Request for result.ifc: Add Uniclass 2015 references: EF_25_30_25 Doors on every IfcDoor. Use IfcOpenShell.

First a look at what the model holds.

```python
import ifcopenshell

model = ifcopenshell.open("result.ifc")
print(model.schema)
print("classifications:", [c.Name for c in model.by_type("IfcClassification")])
for ifc_class in ("IfcDoor", "IfcRoof", "IfcStair", "IfcWall", "IfcWindow"):
    print(ifc_class, len(model.by_type(ifc_class)))
```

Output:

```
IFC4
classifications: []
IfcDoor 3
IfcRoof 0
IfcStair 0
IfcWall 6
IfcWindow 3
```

```python
import ifcopenshell
import ifcopenshell.api.classification

model = ifcopenshell.open("result.ifc")

system = ifcopenshell.api.classification.add_classification(model, classification="Uniclass 2015")

codes = {
    "IfcDoor": ("EF_25_30_25", "Doors"),
}
for ifc_class, (code, name) in codes.items():
    products = model.by_type(ifc_class)
    ifcopenshell.api.classification.add_reference(
        model, products=products, classification=system, identification=code, name=name
    )
    print(code, len(products))

model.write("result_updated.ifc")
```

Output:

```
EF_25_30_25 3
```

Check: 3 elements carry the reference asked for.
